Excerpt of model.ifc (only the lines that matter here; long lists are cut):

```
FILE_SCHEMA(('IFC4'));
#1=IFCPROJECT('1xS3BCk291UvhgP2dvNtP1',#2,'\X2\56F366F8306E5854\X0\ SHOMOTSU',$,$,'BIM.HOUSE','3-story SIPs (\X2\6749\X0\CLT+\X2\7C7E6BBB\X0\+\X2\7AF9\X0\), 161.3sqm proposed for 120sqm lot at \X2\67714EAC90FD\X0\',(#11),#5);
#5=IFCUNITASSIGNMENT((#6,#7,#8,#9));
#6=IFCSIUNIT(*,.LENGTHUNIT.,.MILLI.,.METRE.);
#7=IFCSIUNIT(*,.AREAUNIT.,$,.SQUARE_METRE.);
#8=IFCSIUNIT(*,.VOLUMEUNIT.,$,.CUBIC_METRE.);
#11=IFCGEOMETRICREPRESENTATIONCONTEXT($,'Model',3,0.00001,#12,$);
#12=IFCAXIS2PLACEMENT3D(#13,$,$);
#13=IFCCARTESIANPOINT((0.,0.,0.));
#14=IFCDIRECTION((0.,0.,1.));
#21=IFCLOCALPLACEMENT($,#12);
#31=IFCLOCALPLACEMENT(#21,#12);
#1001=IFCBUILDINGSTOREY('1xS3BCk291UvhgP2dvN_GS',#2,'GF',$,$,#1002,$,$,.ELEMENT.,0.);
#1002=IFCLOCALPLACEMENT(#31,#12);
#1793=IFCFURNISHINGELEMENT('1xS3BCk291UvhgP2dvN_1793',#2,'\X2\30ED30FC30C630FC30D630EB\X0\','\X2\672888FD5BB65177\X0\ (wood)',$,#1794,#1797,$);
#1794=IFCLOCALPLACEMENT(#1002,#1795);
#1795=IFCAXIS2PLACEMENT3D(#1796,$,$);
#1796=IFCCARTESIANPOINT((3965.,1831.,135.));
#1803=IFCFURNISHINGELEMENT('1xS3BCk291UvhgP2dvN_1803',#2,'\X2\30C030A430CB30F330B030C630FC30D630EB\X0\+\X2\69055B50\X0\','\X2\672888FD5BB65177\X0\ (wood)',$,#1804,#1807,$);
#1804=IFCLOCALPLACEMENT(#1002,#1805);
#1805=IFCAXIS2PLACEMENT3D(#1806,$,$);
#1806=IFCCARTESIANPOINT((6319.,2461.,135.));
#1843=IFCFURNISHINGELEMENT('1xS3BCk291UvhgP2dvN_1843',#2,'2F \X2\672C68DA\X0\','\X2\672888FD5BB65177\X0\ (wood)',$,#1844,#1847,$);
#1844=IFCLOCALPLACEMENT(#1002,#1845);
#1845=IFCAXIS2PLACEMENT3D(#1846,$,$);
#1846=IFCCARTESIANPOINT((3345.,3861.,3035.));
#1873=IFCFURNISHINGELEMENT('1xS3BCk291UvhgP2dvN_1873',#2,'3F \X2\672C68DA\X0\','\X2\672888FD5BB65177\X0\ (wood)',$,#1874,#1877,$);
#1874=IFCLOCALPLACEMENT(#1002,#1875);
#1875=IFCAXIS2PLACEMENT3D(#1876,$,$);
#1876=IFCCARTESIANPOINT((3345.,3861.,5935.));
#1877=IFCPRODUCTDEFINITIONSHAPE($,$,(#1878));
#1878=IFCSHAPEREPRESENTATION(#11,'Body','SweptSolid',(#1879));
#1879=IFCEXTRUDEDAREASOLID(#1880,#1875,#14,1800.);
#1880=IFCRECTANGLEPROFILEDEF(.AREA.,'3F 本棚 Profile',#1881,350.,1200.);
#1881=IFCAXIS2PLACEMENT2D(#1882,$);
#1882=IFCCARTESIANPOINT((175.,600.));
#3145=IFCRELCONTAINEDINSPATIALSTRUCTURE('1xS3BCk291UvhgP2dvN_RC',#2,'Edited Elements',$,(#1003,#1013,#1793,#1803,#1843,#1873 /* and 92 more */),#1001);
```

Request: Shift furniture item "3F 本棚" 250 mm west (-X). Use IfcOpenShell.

```python
import ifcopenshell
import ifcopenshell.api.geometry
import ifcopenshell.util.placement
import ifcopenshell.util.unit

model = ifcopenshell.open("model.ifc")
unit_scale = ifcopenshell.util.unit.calculate_unit_scale(model)

item = model.by_guid("1xS3BCk291UvhgP2dvN_1873")
matrix = ifcopenshell.util.placement.get_local_placement(item.ObjectPlacement)
matrix[0, 3] -= 0.25 / unit_scale
ifcopenshell.api.geometry.edit_object_placement(model, product=item, matrix=matrix, is_si=False)

print(ifcopenshell.util.placement.get_local_placement(item.ObjectPlacement).round(3) + 0.0)

model.write("model_rev.ifc")
```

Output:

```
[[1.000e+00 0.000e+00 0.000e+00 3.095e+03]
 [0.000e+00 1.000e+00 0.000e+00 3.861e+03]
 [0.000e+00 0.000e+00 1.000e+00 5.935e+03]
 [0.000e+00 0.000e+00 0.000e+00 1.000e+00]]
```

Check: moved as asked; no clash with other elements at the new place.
